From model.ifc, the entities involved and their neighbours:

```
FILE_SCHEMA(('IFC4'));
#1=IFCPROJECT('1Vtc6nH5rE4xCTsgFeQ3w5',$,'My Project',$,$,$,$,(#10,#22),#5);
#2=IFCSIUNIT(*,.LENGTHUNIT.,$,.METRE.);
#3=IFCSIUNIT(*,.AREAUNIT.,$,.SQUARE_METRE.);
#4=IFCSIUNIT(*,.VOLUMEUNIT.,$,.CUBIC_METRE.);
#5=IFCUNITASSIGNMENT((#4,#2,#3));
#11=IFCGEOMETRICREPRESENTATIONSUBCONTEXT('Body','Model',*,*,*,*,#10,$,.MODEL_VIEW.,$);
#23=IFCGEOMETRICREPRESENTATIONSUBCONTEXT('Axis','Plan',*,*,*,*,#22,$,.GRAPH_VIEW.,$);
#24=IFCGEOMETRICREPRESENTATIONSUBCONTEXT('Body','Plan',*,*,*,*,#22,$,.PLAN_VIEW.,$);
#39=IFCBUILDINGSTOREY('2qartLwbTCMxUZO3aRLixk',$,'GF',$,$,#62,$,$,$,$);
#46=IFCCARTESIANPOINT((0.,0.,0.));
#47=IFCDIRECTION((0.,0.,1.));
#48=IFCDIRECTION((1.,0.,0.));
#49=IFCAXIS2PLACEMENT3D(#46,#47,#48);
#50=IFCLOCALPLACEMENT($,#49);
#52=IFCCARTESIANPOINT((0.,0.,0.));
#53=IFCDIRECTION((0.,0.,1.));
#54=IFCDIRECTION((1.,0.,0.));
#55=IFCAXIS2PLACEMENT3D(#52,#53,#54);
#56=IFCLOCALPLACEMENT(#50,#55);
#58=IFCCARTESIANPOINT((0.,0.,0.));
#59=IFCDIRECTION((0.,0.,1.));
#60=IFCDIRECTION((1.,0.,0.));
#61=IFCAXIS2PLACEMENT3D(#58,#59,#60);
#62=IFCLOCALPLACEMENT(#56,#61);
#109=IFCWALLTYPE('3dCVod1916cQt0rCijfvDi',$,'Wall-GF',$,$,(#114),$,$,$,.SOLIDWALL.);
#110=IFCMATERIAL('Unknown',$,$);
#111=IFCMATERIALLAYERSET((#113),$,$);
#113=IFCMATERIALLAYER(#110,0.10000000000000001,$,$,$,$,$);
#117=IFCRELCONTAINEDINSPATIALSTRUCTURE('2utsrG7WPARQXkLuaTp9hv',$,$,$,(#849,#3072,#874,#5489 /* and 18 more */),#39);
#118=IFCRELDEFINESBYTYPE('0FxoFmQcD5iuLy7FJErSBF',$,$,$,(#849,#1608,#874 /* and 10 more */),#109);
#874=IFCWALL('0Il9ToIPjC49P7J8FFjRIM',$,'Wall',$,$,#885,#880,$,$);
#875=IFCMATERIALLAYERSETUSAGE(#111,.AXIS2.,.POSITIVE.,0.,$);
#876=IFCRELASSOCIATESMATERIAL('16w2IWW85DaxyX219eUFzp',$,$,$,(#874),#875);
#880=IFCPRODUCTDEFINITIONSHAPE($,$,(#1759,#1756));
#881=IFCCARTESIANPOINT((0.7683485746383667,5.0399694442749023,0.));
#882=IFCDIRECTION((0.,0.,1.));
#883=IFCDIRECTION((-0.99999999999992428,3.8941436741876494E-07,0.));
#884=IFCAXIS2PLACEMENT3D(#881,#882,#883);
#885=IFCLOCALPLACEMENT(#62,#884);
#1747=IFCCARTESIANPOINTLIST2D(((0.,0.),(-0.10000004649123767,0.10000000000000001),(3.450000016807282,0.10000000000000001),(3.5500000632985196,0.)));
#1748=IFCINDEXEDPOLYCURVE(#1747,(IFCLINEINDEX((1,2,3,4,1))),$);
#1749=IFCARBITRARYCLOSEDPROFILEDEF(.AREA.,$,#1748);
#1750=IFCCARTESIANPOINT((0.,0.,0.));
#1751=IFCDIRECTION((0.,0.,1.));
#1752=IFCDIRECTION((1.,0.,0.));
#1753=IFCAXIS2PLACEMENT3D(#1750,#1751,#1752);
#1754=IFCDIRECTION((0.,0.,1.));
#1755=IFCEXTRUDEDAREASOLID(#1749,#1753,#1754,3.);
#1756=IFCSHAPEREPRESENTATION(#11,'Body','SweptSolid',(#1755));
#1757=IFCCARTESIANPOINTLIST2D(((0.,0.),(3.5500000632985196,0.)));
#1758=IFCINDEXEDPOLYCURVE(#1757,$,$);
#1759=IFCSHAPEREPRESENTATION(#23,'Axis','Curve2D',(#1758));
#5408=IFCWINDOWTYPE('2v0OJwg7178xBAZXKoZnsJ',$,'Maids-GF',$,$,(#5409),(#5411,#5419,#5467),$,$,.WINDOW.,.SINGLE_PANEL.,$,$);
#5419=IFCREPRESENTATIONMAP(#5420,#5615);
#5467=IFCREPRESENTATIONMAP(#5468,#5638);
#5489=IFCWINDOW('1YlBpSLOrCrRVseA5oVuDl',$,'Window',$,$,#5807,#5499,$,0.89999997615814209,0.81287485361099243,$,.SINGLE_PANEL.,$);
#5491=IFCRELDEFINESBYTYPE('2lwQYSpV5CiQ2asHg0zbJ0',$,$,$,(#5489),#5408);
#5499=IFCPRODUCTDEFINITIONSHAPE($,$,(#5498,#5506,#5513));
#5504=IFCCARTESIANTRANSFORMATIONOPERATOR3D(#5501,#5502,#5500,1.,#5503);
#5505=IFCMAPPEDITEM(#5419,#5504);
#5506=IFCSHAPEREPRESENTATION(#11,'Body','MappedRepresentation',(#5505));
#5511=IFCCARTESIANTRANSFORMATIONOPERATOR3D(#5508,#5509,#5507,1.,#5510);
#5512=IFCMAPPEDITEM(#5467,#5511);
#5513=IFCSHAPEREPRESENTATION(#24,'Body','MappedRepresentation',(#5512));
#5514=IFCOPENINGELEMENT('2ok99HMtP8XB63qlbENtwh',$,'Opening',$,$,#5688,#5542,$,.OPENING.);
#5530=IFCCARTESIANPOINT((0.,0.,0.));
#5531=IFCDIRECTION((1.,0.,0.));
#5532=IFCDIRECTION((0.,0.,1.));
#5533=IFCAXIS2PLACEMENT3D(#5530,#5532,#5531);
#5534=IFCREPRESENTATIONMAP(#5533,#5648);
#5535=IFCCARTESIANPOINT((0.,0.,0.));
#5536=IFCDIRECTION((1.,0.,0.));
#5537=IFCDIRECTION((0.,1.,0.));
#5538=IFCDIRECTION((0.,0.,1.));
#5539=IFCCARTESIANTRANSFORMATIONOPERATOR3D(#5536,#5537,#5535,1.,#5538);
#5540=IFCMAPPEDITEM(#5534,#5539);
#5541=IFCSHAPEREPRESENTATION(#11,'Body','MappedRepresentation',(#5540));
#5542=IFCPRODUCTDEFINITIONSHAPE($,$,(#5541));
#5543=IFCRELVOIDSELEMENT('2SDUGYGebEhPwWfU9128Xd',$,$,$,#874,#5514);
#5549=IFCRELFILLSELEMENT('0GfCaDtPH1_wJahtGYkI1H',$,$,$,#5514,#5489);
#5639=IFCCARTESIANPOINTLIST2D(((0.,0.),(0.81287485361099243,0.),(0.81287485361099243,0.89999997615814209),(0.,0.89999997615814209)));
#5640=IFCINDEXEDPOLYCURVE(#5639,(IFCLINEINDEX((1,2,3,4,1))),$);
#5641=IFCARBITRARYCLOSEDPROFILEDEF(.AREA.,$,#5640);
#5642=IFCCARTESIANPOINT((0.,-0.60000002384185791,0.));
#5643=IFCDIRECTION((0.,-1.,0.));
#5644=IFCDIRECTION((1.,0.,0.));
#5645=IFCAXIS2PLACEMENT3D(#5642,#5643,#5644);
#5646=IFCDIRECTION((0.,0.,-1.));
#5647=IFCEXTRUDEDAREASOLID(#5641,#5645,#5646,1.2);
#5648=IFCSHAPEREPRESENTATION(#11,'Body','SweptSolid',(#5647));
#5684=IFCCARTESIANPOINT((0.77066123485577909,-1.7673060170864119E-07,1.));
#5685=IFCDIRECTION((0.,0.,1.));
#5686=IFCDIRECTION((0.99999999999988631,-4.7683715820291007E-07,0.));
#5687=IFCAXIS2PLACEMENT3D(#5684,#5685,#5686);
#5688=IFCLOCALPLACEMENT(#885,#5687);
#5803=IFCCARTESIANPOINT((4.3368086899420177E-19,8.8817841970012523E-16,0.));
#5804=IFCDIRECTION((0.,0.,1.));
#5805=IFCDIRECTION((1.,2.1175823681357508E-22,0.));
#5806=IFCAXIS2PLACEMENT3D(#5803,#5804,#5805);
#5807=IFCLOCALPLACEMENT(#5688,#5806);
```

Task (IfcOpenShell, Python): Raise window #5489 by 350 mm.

```python
import numpy as np
import ifcopenshell
import ifcopenshell.api.geometry
import ifcopenshell.util.placement
import ifcopenshell.util.unit

model = ifcopenshell.open("model.ifc")
unit_scale = ifcopenshell.util.unit.calculate_unit_scale(model)

window = model.by_guid("1YlBpSLOrCrRVseA5oVuDl")
opening = window.FillsVoids[0].RelatingOpeningElement
dz = 0.35

shift = np.array([0.0, 0.0, dz])
# The window is placed relative to its opening, so it follows when the opening moves.
matrix = ifcopenshell.util.placement.get_local_placement(opening.ObjectPlacement)
matrix[:3, 3] += shift
ifcopenshell.api.geometry.edit_object_placement(
    model, product=opening, matrix=matrix, is_si=False, should_transform_children=True
)

print(f"moved by {dz * unit_scale:+.3f} m")

model.write("model_v2.ifc")
```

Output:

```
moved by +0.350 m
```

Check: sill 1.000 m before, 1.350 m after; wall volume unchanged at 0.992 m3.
